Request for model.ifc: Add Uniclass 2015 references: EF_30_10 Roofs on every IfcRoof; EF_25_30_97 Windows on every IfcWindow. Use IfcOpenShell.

First a look at what the model holds.

```python
import ifcopenshell

model = ifcopenshell.open("model.ifc")
print(model.schema)
print("classifications:", [c.Name for c in model.by_type("IfcClassification")])
for ifc_class in ("IfcDoor", "IfcRoof", "IfcStair", "IfcWall", "IfcWindow"):
    print(ifc_class, len(model.by_type(ifc_class)))
```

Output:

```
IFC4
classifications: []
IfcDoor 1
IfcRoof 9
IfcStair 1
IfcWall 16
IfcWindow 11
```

```python
import ifcopenshell
import ifcopenshell.api.classification

model = ifcopenshell.open("model.ifc")

system = ifcopenshell.api.classification.add_classification(model, classification="Uniclass 2015")

codes = {
    "IfcRoof": ("EF_30_10", "Roofs"),
    "IfcWindow": ("EF_25_30_97", "Windows"),
}
for ifc_class, (code, name) in codes.items():
    products = model.by_type(ifc_class)
    ifcopenshell.api.classification.add_reference(
        model, products=products, classification=system, identification=code, name=name
    )
    print(code, len(products))

model.write("model_updated.ifc")
```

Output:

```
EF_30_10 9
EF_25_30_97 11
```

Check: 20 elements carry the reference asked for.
